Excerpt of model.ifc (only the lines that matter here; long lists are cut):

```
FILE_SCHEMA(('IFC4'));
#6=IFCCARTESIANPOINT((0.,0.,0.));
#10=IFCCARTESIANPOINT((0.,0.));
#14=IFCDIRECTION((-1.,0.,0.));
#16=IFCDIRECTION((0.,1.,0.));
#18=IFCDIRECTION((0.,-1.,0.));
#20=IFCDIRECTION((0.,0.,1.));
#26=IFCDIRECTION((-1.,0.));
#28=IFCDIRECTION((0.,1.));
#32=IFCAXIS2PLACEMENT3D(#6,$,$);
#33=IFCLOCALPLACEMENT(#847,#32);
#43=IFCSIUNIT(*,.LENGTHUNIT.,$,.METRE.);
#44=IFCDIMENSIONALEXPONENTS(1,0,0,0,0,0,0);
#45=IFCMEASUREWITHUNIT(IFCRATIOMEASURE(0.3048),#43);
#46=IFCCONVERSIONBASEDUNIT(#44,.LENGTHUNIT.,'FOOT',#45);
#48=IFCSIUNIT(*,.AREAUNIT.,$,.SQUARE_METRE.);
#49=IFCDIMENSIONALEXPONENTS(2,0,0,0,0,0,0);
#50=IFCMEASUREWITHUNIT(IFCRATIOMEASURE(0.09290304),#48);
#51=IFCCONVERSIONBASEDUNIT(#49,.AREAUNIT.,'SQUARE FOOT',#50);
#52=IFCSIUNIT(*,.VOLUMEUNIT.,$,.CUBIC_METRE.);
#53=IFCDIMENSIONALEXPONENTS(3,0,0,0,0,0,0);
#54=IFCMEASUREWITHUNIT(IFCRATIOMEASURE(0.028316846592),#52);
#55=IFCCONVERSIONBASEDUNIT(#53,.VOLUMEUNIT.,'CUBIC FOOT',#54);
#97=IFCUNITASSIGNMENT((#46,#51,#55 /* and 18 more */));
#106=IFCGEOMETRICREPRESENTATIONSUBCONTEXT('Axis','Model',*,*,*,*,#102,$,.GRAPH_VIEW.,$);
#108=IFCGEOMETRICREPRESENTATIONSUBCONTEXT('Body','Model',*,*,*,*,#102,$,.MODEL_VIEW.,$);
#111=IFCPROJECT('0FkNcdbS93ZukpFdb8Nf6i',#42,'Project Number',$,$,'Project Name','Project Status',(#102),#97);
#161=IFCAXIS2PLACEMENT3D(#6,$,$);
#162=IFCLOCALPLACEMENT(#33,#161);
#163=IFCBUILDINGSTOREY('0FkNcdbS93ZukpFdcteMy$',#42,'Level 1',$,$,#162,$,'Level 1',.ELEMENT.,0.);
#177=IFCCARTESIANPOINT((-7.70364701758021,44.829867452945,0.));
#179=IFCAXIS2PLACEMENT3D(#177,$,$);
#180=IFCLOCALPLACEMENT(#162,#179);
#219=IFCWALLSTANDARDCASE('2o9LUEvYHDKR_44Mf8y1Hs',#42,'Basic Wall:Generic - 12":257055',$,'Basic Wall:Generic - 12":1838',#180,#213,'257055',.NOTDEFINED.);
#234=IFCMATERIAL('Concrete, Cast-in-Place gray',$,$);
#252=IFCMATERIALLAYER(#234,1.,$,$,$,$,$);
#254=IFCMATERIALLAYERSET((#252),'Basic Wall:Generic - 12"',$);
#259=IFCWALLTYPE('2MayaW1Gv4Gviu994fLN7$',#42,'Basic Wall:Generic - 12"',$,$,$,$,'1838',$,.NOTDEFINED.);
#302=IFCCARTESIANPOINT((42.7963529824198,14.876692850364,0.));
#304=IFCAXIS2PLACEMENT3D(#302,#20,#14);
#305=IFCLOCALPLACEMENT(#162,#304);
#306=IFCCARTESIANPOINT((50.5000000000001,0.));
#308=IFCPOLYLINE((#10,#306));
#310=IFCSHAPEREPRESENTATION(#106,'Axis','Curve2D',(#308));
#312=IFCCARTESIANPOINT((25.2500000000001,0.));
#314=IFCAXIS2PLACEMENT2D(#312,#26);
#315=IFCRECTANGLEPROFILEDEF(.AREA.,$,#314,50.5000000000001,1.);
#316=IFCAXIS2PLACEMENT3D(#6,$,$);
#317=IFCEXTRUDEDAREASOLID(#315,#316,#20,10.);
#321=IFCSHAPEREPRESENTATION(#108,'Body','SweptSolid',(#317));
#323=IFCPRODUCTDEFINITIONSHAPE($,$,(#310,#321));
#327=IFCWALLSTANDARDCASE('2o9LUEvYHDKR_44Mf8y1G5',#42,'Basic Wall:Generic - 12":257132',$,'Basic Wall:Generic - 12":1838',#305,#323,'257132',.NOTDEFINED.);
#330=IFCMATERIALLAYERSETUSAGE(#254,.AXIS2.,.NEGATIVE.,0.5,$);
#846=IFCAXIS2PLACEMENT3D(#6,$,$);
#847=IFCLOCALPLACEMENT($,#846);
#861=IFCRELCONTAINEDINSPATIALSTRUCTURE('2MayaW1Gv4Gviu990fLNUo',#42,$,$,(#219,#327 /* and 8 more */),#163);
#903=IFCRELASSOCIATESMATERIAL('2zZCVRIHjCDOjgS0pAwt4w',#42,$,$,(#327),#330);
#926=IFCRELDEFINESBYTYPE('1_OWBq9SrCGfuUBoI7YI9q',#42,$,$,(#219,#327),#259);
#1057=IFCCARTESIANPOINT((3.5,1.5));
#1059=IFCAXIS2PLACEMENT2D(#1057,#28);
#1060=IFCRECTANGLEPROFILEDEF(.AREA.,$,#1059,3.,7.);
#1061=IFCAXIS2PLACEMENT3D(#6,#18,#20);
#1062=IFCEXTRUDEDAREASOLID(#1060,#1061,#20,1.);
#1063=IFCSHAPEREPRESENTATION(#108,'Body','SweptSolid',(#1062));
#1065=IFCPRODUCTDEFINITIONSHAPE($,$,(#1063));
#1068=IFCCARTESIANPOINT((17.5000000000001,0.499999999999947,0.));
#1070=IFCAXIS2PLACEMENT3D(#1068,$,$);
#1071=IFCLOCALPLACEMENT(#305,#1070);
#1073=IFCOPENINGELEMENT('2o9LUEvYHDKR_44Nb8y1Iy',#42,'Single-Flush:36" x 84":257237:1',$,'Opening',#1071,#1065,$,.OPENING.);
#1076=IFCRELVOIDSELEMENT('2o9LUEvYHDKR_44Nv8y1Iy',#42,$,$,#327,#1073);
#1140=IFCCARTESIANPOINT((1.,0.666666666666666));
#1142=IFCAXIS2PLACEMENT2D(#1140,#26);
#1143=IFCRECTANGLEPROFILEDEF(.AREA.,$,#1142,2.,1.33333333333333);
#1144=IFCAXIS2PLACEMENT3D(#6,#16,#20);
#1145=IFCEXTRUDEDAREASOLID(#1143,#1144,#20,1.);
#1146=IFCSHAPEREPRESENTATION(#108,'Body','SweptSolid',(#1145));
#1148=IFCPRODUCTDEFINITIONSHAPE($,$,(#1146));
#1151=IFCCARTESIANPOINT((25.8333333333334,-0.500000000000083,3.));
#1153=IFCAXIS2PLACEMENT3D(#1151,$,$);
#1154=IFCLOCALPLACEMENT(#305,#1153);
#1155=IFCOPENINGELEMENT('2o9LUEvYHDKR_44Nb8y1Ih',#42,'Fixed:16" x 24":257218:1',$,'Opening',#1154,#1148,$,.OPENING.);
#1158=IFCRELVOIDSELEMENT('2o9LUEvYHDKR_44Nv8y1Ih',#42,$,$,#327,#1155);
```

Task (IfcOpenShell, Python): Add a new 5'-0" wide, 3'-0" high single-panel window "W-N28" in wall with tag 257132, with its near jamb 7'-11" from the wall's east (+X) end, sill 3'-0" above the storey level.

```python
import numpy as np
import ifcopenshell
import ifcopenshell.api.feature
import ifcopenshell.api.geometry
import ifcopenshell.api.root
import ifcopenshell.api.spatial
import ifcopenshell.geom
import ifcopenshell.util.element
import ifcopenshell.util.placement
import ifcopenshell.util.representation
import ifcopenshell.util.shape
import ifcopenshell.util.unit

model = ifcopenshell.open("model.ifc")
unit_scale = ifcopenshell.util.unit.calculate_unit_scale(model)
settings = ifcopenshell.geom.settings()


def volume(element):
    """Net volume in cubic metres, openings subtracted."""
    shape = ifcopenshell.geom.create_shape(settings, element)
    return ifcopenshell.util.shape.get_volume(shape.geometry)


wall = model.by_guid("2o9LUEvYHDKR_44Mf8y1G5")
storey = ifcopenshell.util.element.get_container(wall, ifc_class="IfcBuildingStorey")
context = ifcopenshell.util.representation.get_context(model, "Model", "Body", "MODEL_VIEW")
before = volume(wall)

width, height, from_end, sill = 1.524, 0.9144, 2.413, 0.9144  # metres

# The wall runs along its own X axis, and the end named is its -X end.
wall_shape = ifcopenshell.geom.create_shape(settings, wall)
x, y, z = ifcopenshell.util.shape.get_vertices(wall_shape.geometry).T
start = x.min() + from_end
face, thickness = float(y.min()), float(y.max() - y.min())
wall_matrix = ifcopenshell.util.placement.get_local_placement(wall.ObjectPlacement)
level = ifcopenshell.util.placement.get_local_placement(storey.ObjectPlacement)[2, 3]


def in_wall(x, y):
    """Placement at x, y metres in the wall's axes, at sill height."""
    matrix = wall_matrix.copy()
    matrix[:, 3] = wall_matrix @ np.array([x / unit_scale, y / unit_scale, 0.0, 1.0])
    matrix[2, 3] = level + sill / unit_scale
    return matrix


# Opening: a box that overshoots both wall faces by 50 mm.
opening = ifcopenshell.api.root.create_entity(model, ifc_class="IfcOpeningElement", predefined_type="OPENING")
box = ifcopenshell.api.geometry.add_wall_representation(
    model, context=context, length=width, height=height, thickness=thickness + 0.1
)
ifcopenshell.api.geometry.assign_representation(model, product=opening, representation=box)
ifcopenshell.api.geometry.edit_object_placement(model, product=opening, matrix=in_wall(start, face - 0.05), is_si=False)
ifcopenshell.api.feature.add_feature(model, feature=opening, element=wall)

window = ifcopenshell.api.root.create_entity(model, ifc_class="IfcWindow", name="W-N28", predefined_type="WINDOW")
window.OverallWidth, window.OverallHeight = width / unit_scale, height / unit_scale
window.PartitioningType = "SINGLE_PANEL"
body = ifcopenshell.api.geometry.add_window_representation(
    model,
    context=context,
    overall_width=window.OverallWidth,
    overall_height=window.OverallHeight,
    partition_type="SINGLE_PANEL",
)
ifcopenshell.api.geometry.assign_representation(model, product=window, representation=body)
ifcopenshell.api.spatial.assign_container(model, products=[window], relating_structure=storey)
ifcopenshell.api.feature.add_filling(model, opening=opening, element=window)

# Centre the window in the wall's thickness.
ifcopenshell.api.geometry.edit_object_placement(model, product=window, matrix=in_wall(start, face), is_si=False)
window_shape = ifcopenshell.geom.create_shape(settings, window)
depth = ifcopenshell.util.shape.get_vertices(window_shape.geometry)[:, 1]
offset = face + thickness / 2 - (depth.min() + depth.max()) / 2
ifcopenshell.api.geometry.edit_object_placement(model, product=window, matrix=in_wall(start, offset), is_si=False)

after = volume(wall)

print(f"wall volume {before:.3f} -> {after:.3f} m3")

model.write("model_edited.ifc")
```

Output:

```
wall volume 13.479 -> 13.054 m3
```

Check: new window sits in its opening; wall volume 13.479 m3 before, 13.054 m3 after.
